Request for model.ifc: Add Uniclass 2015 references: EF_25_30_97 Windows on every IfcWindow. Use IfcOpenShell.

First a look at what the model holds.

```python
import ifcopenshell

model = ifcopenshell.open("model.ifc")
print(model.schema)
print("classifications:", [c.Name for c in model.by_type("IfcClassification")])
for ifc_class in ("IfcDoor", "IfcRoof", "IfcStair", "IfcWall", "IfcWindow"):
    print(ifc_class, len(model.by_type(ifc_class)))
```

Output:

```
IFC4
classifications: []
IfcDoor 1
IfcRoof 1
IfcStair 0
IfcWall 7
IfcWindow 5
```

```python
import ifcopenshell
import ifcopenshell.api.classification

model = ifcopenshell.open("model.ifc")

system = ifcopenshell.api.classification.add_classification(model, classification="Uniclass 2015")

codes = {
    "IfcWindow": ("EF_25_30_97", "Windows"),
}
for ifc_class, (code, name) in codes.items():
    products = model.by_type(ifc_class)
    ifcopenshell.api.classification.add_reference(
        model, products=products, classification=system, identification=code, name=name
    )
    print(code, len(products))

model.write("model-out.ifc")
```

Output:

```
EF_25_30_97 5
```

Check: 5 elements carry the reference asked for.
